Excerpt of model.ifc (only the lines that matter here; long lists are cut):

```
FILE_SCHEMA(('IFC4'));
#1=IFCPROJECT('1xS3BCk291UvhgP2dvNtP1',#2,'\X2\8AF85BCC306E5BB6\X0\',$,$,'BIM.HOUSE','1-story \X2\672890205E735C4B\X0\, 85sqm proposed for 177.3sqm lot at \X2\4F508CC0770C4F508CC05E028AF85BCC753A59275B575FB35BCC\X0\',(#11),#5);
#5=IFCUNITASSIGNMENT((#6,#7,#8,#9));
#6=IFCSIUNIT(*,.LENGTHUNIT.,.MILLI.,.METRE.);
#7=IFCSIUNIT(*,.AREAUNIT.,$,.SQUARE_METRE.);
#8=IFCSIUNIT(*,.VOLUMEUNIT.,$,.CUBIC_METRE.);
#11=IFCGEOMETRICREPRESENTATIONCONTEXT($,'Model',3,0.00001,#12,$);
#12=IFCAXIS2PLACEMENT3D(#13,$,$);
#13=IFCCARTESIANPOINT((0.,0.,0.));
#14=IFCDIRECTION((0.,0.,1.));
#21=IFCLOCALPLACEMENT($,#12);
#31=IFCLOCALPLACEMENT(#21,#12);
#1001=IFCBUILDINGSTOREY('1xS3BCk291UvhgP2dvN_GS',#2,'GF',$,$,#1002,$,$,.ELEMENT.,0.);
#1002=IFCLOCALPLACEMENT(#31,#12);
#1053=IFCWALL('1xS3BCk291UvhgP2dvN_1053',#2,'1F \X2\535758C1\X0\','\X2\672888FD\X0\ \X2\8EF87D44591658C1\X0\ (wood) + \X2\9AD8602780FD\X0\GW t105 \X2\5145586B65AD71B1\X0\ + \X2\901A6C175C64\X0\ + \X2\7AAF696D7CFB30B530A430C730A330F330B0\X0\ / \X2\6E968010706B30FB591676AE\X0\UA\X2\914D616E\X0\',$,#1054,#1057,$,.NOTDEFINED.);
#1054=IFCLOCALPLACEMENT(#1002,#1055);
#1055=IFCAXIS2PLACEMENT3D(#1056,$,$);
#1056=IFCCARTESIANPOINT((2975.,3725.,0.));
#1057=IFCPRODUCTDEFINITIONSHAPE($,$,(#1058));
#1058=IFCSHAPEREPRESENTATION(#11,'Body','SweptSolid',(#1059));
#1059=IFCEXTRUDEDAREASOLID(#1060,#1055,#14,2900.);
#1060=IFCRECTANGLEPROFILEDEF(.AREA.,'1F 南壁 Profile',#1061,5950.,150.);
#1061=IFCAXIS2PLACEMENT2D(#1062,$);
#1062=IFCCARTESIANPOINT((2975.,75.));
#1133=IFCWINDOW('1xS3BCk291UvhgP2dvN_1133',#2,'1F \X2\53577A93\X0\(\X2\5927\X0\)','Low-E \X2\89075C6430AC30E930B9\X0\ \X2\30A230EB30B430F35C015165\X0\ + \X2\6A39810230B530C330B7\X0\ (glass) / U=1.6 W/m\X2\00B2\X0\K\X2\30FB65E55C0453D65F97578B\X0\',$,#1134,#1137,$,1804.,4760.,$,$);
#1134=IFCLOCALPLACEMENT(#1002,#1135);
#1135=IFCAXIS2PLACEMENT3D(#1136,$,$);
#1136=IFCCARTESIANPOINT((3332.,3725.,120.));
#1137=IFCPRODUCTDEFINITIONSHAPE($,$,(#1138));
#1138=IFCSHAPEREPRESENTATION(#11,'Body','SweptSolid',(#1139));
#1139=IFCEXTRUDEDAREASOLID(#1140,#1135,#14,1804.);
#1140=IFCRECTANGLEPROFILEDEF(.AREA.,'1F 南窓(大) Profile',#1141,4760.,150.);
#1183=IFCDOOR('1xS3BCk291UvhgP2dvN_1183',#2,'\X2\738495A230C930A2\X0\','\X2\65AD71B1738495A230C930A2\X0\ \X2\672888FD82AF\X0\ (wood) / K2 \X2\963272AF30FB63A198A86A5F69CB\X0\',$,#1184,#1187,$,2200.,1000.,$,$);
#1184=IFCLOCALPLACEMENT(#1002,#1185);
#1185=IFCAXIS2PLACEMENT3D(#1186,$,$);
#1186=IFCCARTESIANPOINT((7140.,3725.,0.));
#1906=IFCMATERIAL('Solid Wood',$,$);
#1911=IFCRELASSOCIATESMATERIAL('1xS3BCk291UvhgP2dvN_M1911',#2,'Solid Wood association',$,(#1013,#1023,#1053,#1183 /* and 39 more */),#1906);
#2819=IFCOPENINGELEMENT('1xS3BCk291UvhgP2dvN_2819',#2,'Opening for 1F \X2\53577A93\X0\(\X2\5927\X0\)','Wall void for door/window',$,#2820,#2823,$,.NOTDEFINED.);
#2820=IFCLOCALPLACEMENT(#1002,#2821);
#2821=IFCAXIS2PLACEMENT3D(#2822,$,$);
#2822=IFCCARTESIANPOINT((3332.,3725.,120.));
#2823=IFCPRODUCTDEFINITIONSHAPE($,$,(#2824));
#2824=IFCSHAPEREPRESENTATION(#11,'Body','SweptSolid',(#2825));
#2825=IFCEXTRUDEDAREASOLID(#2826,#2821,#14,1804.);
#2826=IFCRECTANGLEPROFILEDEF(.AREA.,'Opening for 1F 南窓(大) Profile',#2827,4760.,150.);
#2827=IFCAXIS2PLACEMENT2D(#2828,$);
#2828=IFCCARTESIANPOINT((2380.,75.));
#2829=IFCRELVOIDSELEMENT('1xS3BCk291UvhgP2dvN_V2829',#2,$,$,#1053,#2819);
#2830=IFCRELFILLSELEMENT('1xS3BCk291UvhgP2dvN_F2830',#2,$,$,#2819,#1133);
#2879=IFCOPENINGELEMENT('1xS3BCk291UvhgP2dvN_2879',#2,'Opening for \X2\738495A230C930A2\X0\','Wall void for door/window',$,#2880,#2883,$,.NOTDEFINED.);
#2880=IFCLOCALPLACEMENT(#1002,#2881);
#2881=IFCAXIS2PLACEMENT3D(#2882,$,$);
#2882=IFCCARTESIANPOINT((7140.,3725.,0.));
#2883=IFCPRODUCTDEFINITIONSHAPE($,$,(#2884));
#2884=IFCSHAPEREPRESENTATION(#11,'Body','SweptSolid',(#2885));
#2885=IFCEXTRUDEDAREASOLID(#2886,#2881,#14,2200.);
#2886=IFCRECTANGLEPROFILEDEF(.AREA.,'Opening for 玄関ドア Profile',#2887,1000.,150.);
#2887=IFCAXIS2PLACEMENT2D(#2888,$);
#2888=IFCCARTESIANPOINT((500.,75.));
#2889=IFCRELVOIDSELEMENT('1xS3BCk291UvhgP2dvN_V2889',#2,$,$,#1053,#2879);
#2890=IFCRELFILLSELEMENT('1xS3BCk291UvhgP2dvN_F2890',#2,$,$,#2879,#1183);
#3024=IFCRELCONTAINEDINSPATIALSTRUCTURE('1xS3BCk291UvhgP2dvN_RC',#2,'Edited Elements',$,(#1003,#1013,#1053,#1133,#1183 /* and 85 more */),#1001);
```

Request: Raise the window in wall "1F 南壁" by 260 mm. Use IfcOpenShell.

```python
import numpy as np
import ifcopenshell
import ifcopenshell.api.geometry
import ifcopenshell.util.placement
import ifcopenshell.util.unit

model = ifcopenshell.open("model.ifc")
unit_scale = ifcopenshell.util.unit.calculate_unit_scale(model)

window = model.by_guid("1xS3BCk291UvhgP2dvN_1133")
opening = window.FillsVoids[0].RelatingOpeningElement
dz = 260.0

shift = np.array([0.0, 0.0, dz])
# The window is not placed relative to its opening, so move both.
for product in (opening, window):
    matrix = ifcopenshell.util.placement.get_local_placement(product.ObjectPlacement)
    matrix[:3, 3] += shift
    ifcopenshell.api.geometry.edit_object_placement(model, product=product, matrix=matrix, is_si=False)

print(f"moved by {dz * unit_scale:+.3f} m")

model.write("model_v2.ifc")
```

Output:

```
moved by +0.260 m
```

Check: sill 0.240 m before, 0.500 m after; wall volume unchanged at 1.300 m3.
